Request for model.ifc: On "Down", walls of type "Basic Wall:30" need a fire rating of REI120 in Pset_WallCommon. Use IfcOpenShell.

First a look at what the model holds.

```python
import ifcopenshell
import ifcopenshell.util.element

model = ifcopenshell.open("model.ifc")
print(model.schema)
storey = next(s for s in model.by_type("IfcBuildingStorey") if s.Name == "Down")
walls = [e for e in ifcopenshell.util.element.get_decomposition(storey) if e.is_a("IfcWall")]
seen = {}
for e in walls:
    element_type = ifcopenshell.util.element.get_type(e)
    key = (element_type.Name if element_type != e and element_type else None, ifcopenshell.util.element.get_pset(e, "Pset_WallCommon", "FireRating"))
    seen[key] = seen.get(key, 0) + 1
for (name, value), count in sorted(seen.items(), key=str):
    print(count, "x", name, "|", value)
```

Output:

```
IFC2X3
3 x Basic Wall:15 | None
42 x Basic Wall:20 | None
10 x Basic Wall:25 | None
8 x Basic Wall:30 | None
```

```python
import ifcopenshell
import ifcopenshell.api.pset
import ifcopenshell.util.element

model = ifcopenshell.open("model.ifc")

storey = next(s for s in model.by_type("IfcBuildingStorey") if s.Name == "Down")
walls = [e for e in ifcopenshell.util.element.get_decomposition(storey) if e.is_a("IfcWall")]

count = 0
for e in walls:
    element_type = ifcopenshell.util.element.get_type(e)
    if element_type in (None, e) or element_type.Name != "Basic Wall:30":
        continue
    # add_pset returns the element's existing set when there is one.
    pset = ifcopenshell.api.pset.add_pset(model, product=e, name="Pset_WallCommon")
    ifcopenshell.api.pset.edit_pset(model, pset=pset, properties={"FireRating": "REI120"})
    count += 1

print(count, "walls updated")

model.write("model_edited.ifc")
```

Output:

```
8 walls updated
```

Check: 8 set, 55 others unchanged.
